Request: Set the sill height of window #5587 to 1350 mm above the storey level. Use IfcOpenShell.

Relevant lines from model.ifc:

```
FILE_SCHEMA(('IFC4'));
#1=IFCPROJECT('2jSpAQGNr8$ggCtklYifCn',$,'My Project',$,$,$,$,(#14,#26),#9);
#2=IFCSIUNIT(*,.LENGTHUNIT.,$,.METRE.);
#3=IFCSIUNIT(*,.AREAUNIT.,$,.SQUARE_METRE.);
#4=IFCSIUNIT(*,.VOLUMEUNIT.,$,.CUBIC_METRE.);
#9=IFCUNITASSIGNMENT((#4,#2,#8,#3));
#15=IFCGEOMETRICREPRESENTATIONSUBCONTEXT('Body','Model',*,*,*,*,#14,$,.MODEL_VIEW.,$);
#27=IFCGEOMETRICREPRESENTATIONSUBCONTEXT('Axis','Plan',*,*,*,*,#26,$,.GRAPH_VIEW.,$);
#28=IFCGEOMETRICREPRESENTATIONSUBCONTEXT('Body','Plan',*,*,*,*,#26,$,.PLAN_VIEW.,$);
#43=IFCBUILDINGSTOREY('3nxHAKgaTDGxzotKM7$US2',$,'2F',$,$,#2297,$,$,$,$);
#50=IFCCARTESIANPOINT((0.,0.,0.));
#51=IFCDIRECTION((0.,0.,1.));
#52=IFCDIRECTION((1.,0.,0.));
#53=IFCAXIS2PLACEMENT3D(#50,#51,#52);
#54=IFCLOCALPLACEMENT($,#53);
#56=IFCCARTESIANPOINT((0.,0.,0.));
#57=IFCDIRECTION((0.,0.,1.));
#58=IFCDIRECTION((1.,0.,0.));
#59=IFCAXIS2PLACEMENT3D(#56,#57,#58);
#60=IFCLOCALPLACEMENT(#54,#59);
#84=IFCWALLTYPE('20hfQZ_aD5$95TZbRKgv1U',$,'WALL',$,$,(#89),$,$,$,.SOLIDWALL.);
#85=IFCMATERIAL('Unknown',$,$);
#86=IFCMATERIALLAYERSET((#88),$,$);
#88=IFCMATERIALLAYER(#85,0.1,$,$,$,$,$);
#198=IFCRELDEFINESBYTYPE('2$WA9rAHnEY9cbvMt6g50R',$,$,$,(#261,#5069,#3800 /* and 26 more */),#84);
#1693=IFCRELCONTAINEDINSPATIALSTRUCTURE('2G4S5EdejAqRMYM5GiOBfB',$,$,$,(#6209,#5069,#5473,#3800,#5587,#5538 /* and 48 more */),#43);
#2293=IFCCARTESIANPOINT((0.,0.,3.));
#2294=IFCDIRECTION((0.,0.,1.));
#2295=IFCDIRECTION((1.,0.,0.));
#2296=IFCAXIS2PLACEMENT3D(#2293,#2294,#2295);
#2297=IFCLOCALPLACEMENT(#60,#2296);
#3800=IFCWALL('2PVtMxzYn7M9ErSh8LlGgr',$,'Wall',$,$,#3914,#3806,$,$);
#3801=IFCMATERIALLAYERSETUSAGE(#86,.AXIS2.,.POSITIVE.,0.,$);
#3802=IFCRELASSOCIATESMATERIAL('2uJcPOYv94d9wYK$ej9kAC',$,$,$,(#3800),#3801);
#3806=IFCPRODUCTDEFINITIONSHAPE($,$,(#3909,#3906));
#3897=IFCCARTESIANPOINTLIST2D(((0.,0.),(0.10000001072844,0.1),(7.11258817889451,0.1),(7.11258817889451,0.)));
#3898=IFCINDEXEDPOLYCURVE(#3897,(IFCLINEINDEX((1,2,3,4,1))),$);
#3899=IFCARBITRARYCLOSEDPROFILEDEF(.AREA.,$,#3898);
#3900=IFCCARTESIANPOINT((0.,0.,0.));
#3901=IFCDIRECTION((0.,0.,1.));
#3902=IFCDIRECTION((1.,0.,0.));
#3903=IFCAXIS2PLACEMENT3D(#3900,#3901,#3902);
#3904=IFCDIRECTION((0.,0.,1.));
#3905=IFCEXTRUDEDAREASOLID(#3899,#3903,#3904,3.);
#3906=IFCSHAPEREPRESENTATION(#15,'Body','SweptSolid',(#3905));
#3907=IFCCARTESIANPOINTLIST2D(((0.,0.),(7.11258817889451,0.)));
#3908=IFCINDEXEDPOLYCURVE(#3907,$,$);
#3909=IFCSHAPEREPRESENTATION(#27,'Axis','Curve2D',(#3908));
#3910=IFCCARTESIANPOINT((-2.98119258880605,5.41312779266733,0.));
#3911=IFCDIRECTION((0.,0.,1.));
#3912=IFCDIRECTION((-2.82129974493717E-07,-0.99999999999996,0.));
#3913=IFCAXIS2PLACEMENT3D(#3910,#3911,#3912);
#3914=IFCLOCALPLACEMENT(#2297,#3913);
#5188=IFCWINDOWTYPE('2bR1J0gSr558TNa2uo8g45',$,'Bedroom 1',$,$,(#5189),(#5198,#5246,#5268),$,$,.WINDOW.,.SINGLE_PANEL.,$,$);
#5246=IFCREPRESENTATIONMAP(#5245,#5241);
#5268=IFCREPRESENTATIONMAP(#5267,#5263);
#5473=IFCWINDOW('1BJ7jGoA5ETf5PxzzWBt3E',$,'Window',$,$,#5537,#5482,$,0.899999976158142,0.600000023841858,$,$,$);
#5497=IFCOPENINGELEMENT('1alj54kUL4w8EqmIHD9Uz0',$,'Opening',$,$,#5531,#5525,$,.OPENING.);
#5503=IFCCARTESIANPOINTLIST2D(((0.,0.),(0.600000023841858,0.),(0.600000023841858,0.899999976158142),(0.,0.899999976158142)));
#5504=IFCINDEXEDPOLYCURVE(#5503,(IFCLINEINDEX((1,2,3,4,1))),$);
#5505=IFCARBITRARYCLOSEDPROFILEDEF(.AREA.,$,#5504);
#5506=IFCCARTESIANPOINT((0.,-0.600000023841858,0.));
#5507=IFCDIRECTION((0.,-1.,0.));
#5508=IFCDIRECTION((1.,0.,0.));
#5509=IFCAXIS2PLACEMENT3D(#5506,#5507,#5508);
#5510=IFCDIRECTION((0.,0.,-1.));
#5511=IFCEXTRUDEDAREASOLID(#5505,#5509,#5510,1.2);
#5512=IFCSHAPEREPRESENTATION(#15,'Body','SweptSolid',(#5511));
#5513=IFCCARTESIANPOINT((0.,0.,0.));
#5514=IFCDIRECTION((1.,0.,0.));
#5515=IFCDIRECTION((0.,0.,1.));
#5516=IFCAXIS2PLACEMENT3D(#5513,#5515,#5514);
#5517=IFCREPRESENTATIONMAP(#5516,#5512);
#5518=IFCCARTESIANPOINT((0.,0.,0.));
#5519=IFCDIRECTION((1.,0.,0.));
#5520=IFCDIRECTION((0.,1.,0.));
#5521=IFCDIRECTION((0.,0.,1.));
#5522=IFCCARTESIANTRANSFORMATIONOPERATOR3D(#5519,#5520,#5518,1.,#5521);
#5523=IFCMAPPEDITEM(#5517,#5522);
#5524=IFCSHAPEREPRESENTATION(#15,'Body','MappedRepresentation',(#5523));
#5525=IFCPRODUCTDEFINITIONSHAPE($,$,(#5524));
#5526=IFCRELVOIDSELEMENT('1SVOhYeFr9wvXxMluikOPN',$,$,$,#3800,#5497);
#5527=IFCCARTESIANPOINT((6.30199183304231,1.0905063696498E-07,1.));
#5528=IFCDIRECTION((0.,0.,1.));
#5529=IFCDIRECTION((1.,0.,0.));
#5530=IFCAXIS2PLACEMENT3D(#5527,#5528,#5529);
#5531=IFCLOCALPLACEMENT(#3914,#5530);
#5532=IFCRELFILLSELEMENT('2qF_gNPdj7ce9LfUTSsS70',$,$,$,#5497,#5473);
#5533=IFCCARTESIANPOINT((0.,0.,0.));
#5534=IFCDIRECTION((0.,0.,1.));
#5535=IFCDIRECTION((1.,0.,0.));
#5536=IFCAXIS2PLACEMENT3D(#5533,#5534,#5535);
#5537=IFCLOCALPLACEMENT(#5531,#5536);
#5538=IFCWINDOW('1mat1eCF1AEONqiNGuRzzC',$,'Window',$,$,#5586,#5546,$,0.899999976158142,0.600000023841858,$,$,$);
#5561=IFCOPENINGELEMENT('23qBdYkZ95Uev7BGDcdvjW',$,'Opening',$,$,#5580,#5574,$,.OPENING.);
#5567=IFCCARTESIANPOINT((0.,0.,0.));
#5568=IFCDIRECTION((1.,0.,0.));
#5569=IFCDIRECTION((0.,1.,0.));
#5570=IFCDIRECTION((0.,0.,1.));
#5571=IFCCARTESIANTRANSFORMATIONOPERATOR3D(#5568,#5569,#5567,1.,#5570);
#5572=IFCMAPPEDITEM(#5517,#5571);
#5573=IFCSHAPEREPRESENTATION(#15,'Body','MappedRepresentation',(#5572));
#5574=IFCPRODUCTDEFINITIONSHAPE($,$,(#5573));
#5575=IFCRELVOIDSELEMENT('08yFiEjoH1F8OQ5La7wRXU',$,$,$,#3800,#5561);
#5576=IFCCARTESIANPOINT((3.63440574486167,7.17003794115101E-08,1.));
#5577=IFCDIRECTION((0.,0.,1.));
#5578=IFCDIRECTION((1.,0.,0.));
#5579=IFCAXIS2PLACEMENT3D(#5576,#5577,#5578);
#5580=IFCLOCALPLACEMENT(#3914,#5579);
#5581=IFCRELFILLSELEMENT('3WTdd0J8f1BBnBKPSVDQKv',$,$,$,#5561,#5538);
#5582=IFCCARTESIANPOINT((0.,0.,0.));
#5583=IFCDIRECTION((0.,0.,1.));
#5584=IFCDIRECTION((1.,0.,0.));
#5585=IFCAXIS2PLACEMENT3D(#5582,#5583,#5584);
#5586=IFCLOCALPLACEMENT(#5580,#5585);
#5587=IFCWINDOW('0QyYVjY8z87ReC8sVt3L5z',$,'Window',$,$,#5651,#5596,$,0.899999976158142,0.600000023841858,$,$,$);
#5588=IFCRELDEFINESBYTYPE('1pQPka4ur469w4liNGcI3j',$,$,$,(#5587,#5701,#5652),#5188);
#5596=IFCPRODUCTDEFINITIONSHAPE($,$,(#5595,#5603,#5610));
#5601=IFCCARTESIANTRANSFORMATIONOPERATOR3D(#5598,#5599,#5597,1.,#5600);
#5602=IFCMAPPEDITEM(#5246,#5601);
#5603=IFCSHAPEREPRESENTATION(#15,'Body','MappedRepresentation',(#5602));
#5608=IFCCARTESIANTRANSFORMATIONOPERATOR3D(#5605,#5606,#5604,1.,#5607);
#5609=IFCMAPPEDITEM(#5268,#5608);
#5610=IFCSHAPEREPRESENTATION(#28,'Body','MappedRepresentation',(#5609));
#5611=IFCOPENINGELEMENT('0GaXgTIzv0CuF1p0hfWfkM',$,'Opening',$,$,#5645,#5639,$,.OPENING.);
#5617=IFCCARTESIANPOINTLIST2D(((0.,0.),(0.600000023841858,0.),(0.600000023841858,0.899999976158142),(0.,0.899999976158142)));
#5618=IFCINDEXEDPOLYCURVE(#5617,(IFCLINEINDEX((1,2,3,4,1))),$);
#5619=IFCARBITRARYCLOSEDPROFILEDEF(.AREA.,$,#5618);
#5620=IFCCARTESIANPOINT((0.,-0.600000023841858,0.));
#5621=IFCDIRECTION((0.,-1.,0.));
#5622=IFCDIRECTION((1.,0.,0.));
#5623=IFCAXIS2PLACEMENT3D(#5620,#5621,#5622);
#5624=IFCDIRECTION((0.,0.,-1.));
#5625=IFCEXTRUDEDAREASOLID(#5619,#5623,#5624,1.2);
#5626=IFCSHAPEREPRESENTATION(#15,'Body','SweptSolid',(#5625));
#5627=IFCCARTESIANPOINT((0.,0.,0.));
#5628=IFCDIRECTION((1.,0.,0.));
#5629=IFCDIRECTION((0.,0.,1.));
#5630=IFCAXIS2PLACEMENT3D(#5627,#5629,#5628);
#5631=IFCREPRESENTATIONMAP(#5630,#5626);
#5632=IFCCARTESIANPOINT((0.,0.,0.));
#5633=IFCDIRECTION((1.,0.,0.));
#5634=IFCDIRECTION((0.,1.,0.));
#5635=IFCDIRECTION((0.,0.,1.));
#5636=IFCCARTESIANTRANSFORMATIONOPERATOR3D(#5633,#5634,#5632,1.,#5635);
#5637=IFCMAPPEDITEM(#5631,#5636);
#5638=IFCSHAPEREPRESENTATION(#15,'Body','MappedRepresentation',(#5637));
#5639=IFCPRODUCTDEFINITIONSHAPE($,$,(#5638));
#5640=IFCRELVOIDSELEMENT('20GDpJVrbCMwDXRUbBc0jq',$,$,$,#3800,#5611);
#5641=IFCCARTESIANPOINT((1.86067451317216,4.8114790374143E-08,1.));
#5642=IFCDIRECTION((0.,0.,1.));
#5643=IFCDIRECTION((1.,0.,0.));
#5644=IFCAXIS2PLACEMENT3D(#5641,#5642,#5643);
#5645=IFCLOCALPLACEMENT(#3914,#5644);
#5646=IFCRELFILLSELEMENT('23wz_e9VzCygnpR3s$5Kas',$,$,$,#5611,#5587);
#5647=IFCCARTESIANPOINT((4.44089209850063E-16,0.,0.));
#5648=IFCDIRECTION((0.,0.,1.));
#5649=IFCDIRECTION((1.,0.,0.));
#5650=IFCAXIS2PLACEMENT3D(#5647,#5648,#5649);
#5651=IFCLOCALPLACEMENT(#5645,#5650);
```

```python
import numpy as np
import ifcopenshell
import ifcopenshell.api.geometry
import ifcopenshell.geom
import ifcopenshell.util.element
import ifcopenshell.util.placement
import ifcopenshell.util.shape
import ifcopenshell.util.unit

model = ifcopenshell.open("model.ifc")
unit_scale = ifcopenshell.util.unit.calculate_unit_scale(model)

window = model.by_guid("0QyYVjY8z87ReC8sVt3L5z")
opening = window.FillsVoids[0].RelatingOpeningElement
storey = ifcopenshell.util.element.get_container(window, ifc_class="IfcBuildingStorey")
level = ifcopenshell.util.placement.get_local_placement(storey.ObjectPlacement)[2, 3]

# The opening's origin need not be at the sill, so measure its lowest point.
shape = ifcopenshell.geom.create_shape(ifcopenshell.geom.settings(), opening)
bottom = ifcopenshell.util.shape.get_shape_bottom_elevation(shape, shape.geometry) / unit_scale
dz = level + 1.35 - bottom

shift = np.array([0.0, 0.0, dz])
# The window is placed relative to its opening, so it follows when the opening moves.
matrix = ifcopenshell.util.placement.get_local_placement(opening.ObjectPlacement)
matrix[:3, 3] += shift
ifcopenshell.api.geometry.edit_object_placement(
    model, product=opening, matrix=matrix, is_si=False, should_transform_children=True
)

print(f"moved by {dz * unit_scale:+.3f} m")

model.write("model-out.ifc")
```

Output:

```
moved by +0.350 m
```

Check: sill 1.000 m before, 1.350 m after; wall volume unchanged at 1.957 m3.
